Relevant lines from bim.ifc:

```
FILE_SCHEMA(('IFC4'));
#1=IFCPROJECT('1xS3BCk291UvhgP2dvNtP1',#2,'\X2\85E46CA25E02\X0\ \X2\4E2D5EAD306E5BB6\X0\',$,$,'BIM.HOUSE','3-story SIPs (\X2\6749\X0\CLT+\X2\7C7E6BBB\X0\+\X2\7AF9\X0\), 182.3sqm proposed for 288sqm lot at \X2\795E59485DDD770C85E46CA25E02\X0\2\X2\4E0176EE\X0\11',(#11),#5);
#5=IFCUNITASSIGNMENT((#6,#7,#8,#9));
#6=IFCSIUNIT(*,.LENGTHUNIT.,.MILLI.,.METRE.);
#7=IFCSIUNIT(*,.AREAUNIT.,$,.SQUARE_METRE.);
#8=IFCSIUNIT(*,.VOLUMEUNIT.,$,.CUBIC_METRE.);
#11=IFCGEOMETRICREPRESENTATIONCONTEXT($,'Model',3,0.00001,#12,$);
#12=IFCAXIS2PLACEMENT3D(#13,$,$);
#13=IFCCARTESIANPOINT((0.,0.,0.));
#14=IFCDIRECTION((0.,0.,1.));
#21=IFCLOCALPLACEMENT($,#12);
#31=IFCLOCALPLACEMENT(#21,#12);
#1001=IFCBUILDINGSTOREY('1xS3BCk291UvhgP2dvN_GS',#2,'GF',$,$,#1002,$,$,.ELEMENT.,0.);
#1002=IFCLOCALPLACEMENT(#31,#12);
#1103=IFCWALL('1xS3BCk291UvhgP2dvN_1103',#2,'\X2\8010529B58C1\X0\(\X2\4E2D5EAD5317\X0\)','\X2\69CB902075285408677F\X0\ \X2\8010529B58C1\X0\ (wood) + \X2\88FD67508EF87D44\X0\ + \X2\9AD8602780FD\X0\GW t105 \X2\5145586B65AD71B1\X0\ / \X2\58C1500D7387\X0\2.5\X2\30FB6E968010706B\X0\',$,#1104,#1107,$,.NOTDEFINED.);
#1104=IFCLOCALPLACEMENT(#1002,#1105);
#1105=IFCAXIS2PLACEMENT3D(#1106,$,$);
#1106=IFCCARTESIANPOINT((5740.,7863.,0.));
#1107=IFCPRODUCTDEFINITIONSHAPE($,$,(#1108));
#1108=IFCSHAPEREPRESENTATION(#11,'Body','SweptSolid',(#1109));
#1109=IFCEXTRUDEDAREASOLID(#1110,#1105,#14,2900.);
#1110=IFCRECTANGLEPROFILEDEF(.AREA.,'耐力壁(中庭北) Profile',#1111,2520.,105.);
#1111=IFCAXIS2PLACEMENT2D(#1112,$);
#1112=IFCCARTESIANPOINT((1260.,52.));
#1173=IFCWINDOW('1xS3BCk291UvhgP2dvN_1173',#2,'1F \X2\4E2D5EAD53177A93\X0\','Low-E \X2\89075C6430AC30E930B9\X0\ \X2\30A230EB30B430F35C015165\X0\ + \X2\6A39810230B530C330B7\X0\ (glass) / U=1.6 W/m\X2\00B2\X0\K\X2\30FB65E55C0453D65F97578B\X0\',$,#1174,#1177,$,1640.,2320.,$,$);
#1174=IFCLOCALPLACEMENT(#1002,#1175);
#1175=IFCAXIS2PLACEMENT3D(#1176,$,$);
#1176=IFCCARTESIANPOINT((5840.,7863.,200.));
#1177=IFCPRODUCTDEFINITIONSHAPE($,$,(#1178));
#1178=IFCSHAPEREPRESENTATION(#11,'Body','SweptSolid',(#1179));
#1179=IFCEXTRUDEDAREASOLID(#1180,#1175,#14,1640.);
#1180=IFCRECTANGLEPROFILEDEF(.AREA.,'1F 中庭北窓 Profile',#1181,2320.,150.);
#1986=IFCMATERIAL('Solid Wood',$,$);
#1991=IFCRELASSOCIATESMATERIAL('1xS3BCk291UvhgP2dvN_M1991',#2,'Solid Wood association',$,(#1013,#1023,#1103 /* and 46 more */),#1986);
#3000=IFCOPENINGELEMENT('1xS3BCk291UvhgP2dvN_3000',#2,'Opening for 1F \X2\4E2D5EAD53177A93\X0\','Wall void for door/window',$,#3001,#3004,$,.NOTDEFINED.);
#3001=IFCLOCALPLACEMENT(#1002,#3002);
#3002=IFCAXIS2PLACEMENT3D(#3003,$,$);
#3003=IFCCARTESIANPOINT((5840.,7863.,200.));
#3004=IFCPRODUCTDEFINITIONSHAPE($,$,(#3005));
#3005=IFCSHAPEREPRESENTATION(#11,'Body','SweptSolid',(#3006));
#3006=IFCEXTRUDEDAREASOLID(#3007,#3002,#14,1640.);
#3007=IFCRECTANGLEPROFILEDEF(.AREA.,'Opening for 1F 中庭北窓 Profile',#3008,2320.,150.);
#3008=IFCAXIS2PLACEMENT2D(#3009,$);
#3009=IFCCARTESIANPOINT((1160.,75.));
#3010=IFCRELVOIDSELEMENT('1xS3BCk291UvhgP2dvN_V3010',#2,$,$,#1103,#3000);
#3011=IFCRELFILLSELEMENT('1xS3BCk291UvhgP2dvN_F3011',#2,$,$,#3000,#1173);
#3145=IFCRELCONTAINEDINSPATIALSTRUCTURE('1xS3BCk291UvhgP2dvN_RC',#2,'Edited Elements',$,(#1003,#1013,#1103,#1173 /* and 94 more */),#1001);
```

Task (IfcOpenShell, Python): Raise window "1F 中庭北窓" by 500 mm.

```python
import numpy as np
import ifcopenshell
import ifcopenshell.api.geometry
import ifcopenshell.util.placement
import ifcopenshell.util.unit

model = ifcopenshell.open("bim.ifc")
unit_scale = ifcopenshell.util.unit.calculate_unit_scale(model)

window = model.by_id(1173)
opening = window.FillsVoids[0].RelatingOpeningElement
dz = 500.0

shift = np.array([0.0, 0.0, dz])
# The window is not placed relative to its opening, so move both.
for product in (opening, window):
    matrix = ifcopenshell.util.placement.get_local_placement(product.ObjectPlacement)
    matrix[:3, 3] += shift
    ifcopenshell.api.geometry.edit_object_placement(model, product=product, matrix=matrix, is_si=False)

print(f"moved by {dz * unit_scale:+.3f} m")

model.write("bim-out.ifc")
```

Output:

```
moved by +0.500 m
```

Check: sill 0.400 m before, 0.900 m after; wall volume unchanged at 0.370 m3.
